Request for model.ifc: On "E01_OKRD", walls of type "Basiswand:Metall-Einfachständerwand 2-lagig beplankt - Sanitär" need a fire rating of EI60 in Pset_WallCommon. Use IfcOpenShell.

First a look at what the model holds.

```python
import ifcopenshell
import ifcopenshell.util.element

model = ifcopenshell.open("model.ifc")
print(model.schema)
storey = next(s for s in model.by_type("IfcBuildingStorey") if s.Name == "E01_OKRD")
walls = [e for e in ifcopenshell.util.element.get_decomposition(storey) if e.is_a("IfcWall")]
seen = {}
for e in walls:
    element_type = ifcopenshell.util.element.get_type(e)
    key = (element_type.Name if element_type != e and element_type else None, ifcopenshell.util.element.get_pset(e, "Pset_WallCommon", "FireRating"))
    seen[key] = seen.get(key, 0) + 1
for (name, value), count in sorted(seen.items(), key=str):
    print(count, "x", name, "|", value)
```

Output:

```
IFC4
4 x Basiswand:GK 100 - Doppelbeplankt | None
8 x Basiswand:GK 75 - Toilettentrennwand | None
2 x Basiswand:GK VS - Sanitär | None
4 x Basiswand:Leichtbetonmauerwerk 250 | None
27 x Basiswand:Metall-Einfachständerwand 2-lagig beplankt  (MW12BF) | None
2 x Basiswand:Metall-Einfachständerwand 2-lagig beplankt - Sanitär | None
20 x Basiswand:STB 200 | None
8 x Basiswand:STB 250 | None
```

```python
import ifcopenshell
import ifcopenshell.api.pset
import ifcopenshell.util.element

model = ifcopenshell.open("model.ifc")

storey = next(s for s in model.by_type("IfcBuildingStorey") if s.Name == "E01_OKRD")
walls = [e for e in ifcopenshell.util.element.get_decomposition(storey) if e.is_a("IfcWall")]

count = 0
for e in walls:
    element_type = ifcopenshell.util.element.get_type(e)
    if element_type in (None, e) or element_type.Name != "Basiswand:Metall-Einfachständerwand 2-lagig beplankt - Sanitär":
        continue
    # add_pset returns the element's existing set when there is one.
    pset = ifcopenshell.api.pset.add_pset(model, product=e, name="Pset_WallCommon")
    ifcopenshell.api.pset.edit_pset(model, pset=pset, properties={"FireRating": "EI60"})
    count += 1

print(count, "walls updated")

model.write("model_rev.ifc")
```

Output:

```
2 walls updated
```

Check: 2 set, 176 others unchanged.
